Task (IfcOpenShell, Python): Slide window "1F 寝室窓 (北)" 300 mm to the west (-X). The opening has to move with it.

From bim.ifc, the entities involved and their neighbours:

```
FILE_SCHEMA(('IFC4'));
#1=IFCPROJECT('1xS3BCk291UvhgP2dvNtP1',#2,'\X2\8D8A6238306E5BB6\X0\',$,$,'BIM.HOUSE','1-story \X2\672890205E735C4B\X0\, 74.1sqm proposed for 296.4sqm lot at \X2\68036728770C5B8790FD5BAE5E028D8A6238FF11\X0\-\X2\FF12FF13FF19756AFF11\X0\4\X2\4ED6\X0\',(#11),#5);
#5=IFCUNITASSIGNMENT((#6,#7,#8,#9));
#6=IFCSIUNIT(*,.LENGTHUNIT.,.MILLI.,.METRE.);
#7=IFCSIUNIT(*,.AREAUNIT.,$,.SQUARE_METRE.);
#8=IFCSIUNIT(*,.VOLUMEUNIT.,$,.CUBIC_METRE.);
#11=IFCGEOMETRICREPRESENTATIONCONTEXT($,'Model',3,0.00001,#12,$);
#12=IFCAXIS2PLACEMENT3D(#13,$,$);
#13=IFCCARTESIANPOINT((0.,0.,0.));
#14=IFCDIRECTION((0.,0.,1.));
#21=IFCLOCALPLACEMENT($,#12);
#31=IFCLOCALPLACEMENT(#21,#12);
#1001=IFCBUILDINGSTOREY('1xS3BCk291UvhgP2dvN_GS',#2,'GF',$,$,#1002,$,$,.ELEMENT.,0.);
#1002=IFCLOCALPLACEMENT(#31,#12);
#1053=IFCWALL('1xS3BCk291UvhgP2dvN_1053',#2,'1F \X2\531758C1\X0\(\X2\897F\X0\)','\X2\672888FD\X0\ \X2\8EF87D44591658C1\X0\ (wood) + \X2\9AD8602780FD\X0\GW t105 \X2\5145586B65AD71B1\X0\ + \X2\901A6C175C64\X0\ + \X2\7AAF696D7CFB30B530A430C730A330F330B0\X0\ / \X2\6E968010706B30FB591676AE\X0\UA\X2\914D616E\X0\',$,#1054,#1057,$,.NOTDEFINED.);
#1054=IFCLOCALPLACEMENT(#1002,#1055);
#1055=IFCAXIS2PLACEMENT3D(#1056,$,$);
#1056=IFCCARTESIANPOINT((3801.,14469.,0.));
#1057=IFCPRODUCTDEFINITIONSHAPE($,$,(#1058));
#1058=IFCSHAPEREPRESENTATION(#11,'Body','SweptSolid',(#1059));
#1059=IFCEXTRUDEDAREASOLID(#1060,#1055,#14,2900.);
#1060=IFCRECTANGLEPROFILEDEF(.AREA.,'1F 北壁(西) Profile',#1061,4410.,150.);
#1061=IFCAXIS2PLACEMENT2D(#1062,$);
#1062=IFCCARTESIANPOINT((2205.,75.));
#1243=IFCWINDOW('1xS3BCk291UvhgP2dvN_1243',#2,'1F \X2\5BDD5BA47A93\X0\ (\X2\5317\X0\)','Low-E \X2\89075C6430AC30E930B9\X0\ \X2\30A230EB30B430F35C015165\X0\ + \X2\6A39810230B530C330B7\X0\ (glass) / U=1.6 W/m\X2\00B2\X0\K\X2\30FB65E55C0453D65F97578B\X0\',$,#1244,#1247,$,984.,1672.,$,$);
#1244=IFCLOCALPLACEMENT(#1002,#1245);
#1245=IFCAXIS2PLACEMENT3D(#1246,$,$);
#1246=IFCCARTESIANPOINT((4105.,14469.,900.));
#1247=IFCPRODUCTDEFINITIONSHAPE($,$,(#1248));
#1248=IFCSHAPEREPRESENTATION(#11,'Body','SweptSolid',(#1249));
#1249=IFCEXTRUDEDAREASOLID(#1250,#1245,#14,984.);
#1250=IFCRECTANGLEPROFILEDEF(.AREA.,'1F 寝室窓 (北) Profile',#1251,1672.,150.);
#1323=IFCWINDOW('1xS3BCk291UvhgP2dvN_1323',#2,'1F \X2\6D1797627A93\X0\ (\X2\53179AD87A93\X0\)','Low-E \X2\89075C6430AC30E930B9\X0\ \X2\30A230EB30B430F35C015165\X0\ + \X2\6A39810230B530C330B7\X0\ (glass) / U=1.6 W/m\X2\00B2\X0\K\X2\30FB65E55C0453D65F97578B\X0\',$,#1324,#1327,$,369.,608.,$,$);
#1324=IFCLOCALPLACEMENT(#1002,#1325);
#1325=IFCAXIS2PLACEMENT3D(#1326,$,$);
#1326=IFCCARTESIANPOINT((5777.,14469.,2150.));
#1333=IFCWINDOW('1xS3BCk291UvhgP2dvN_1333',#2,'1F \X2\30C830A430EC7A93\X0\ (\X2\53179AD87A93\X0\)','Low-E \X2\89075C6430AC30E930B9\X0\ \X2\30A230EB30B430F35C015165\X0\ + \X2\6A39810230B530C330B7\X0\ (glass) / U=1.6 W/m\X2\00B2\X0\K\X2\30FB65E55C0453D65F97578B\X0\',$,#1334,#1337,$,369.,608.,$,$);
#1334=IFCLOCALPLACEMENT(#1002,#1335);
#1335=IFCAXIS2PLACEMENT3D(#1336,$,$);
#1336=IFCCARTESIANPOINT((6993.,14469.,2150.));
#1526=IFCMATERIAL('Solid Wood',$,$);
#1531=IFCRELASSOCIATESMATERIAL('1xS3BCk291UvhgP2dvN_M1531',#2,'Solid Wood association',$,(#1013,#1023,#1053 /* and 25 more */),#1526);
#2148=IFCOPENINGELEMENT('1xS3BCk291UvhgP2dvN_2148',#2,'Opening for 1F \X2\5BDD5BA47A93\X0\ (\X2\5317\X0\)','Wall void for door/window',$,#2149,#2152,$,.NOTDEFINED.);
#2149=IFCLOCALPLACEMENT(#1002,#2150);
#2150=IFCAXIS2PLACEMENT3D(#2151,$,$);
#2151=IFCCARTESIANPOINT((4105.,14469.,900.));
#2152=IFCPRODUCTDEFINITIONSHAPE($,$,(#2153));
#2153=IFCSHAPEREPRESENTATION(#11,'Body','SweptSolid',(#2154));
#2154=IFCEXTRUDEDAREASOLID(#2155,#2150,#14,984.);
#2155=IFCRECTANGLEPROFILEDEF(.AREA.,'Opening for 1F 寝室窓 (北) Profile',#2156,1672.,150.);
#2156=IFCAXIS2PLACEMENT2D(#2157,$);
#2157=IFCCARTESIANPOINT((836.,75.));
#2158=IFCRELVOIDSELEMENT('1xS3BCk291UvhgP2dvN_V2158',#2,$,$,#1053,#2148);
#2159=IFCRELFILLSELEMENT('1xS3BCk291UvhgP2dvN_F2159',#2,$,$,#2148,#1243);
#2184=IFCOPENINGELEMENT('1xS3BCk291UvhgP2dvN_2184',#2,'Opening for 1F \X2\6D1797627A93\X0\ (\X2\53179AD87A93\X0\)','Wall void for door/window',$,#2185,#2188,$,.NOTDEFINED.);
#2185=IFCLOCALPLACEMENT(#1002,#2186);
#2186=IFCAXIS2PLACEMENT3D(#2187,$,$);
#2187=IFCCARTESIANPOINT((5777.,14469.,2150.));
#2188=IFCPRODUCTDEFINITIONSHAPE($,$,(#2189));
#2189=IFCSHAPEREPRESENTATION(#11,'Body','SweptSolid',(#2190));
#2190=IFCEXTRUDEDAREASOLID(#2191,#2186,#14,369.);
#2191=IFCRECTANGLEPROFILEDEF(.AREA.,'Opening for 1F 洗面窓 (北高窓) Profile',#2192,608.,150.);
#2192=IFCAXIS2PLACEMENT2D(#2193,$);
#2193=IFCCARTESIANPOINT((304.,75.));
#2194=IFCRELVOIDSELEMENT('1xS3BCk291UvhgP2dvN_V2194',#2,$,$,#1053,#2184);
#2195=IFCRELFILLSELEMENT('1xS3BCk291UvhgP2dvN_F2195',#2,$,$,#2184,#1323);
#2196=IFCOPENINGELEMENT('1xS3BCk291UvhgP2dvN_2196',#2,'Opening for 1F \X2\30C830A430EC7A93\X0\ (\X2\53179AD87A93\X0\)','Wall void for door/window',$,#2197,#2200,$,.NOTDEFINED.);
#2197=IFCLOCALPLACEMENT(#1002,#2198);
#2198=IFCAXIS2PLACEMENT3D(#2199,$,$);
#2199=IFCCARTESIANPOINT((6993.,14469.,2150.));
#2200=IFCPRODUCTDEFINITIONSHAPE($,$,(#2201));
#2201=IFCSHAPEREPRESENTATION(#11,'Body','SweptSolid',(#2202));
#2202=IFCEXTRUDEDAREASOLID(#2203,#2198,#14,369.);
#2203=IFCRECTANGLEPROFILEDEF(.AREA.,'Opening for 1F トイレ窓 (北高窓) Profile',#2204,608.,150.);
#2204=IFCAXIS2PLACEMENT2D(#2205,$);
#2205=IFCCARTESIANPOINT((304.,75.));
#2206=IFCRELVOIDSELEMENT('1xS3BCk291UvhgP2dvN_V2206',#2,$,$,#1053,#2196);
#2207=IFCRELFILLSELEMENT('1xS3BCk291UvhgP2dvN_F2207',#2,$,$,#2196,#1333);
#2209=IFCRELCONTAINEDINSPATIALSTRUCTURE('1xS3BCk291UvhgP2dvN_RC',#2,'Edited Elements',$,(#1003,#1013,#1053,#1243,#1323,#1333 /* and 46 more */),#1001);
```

```python
import ifcopenshell
import ifcopenshell.api.geometry
import ifcopenshell.util.placement

model = ifcopenshell.open("bim.ifc")

window = model.by_guid("1xS3BCk291UvhgP2dvN_1243")
opening = window.FillsVoids[0].RelatingOpeningElement
wall = opening.VoidsElements[0].RelatingBuildingElement

wall_matrix = ifcopenshell.util.placement.get_local_placement(wall.ObjectPlacement)
shift = wall_matrix[:3, 0] * -300.0
before = ifcopenshell.util.placement.get_local_placement(window.ObjectPlacement)[:3, 3].copy()

# The window is not placed relative to its opening, so move both.
for product in (opening, window):
    matrix = ifcopenshell.util.placement.get_local_placement(product.ObjectPlacement)
    matrix[:3, 3] += shift
    ifcopenshell.api.geometry.edit_object_placement(model, product=product, matrix=matrix, is_si=False)

after = ifcopenshell.util.placement.get_local_placement(window.ObjectPlacement)[:3, 3]
print("window moved by", (after - before).round(3) + 0.0)

model.write("bim_rev.ifc")
```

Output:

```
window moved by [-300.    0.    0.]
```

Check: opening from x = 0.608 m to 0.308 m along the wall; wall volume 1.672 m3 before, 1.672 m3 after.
